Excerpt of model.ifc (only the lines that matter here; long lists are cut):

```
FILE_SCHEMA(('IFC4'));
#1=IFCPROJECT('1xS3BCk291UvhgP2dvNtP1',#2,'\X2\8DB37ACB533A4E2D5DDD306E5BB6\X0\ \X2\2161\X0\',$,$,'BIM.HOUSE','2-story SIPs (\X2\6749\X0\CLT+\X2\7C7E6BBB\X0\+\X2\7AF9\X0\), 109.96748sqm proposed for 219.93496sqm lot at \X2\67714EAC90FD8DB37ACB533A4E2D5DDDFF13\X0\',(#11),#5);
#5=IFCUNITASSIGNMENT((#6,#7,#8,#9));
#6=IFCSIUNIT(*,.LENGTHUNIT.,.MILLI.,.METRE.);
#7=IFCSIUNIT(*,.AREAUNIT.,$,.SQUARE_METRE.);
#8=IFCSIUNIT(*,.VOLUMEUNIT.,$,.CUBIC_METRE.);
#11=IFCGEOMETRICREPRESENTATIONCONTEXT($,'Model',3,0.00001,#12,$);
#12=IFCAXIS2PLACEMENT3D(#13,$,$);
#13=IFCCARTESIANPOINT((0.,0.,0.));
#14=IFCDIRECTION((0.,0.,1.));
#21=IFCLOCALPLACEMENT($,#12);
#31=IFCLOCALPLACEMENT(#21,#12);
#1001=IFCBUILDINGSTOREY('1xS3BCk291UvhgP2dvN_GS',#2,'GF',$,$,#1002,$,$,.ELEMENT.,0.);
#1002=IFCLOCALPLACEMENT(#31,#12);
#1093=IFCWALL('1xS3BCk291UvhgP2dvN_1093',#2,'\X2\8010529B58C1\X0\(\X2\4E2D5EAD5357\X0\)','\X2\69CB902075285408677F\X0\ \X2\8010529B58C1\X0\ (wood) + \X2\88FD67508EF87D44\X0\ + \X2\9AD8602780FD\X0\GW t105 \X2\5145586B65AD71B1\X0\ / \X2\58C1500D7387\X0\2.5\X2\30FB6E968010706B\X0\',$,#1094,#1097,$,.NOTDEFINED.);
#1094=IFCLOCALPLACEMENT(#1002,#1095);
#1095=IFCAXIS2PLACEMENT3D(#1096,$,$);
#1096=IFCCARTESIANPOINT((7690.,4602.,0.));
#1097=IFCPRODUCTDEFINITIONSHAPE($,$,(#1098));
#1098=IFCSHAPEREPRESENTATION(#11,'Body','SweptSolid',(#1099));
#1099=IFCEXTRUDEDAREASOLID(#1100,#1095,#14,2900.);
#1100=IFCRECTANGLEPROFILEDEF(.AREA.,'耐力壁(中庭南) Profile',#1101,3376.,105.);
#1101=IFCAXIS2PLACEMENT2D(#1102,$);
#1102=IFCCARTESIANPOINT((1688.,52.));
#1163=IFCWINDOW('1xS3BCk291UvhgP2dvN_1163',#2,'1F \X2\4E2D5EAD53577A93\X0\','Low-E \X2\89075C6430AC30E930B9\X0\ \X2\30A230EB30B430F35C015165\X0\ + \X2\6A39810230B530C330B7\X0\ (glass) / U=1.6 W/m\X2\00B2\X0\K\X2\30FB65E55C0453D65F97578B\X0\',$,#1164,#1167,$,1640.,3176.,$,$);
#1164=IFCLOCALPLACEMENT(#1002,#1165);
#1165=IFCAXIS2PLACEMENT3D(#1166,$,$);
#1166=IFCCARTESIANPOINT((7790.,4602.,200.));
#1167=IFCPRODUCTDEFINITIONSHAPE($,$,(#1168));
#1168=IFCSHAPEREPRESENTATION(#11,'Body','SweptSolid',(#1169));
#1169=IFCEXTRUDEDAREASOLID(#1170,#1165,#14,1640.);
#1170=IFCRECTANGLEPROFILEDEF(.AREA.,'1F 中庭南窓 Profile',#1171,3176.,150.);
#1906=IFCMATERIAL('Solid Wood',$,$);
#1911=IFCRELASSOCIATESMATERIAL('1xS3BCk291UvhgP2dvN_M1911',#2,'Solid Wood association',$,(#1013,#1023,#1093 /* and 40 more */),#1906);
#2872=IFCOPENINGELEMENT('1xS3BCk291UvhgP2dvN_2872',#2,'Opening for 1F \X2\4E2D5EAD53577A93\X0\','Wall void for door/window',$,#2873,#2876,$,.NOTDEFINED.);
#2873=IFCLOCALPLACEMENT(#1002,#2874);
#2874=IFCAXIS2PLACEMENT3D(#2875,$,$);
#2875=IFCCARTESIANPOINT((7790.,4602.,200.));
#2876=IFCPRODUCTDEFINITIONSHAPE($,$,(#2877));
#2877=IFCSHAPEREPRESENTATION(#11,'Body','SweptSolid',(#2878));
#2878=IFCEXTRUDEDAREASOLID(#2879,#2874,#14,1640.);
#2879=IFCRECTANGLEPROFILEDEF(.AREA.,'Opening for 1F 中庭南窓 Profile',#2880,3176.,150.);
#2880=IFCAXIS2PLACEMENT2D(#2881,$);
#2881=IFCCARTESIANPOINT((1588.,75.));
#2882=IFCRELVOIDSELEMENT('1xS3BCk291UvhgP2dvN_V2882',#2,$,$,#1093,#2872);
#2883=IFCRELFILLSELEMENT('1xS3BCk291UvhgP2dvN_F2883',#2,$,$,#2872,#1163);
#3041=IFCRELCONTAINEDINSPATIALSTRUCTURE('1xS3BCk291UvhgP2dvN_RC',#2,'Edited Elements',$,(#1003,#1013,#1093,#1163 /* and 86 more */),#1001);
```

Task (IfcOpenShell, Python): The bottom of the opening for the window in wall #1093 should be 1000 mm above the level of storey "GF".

```python
import numpy as np
import ifcopenshell
import ifcopenshell.api.geometry
import ifcopenshell.geom
import ifcopenshell.util.element
import ifcopenshell.util.placement
import ifcopenshell.util.shape
import ifcopenshell.util.unit

model = ifcopenshell.open("model.ifc")
unit_scale = ifcopenshell.util.unit.calculate_unit_scale(model)

window = model.by_id(1163)
opening = window.FillsVoids[0].RelatingOpeningElement
storey = ifcopenshell.util.element.get_container(window, ifc_class="IfcBuildingStorey")
level = ifcopenshell.util.placement.get_local_placement(storey.ObjectPlacement)[2, 3]

# The opening's origin need not be at the sill, so measure its lowest point.
shape = ifcopenshell.geom.create_shape(ifcopenshell.geom.settings(), opening)
bottom = ifcopenshell.util.shape.get_shape_bottom_elevation(shape, shape.geometry) / unit_scale
dz = level + 1 / unit_scale - bottom

shift = np.array([0.0, 0.0, dz])
# The window is not placed relative to its opening, so move both.
for product in (opening, window):
    matrix = ifcopenshell.util.placement.get_local_placement(product.ObjectPlacement)
    matrix[:3, 3] += shift
    ifcopenshell.api.geometry.edit_object_placement(model, product=product, matrix=matrix, is_si=False)

print(f"moved by {dz * unit_scale:+.3f} m")

model.write("model_edited.ifc")
```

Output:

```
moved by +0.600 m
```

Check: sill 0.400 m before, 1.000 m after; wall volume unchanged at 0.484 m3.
